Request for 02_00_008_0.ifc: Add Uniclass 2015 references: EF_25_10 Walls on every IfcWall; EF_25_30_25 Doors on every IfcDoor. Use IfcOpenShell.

First a look at what the model holds.

```python
import ifcopenshell

model = ifcopenshell.open("02_00_008_0.ifc")
print(model.schema)
print("classifications:", [c.Name for c in model.by_type("IfcClassification")])
for ifc_class in ("IfcDoor", "IfcRoof", "IfcStair", "IfcWall", "IfcWindow"):
    print(ifc_class, len(model.by_type(ifc_class)))
```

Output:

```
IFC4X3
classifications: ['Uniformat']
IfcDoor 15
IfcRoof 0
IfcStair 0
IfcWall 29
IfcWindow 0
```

```python
import ifcopenshell
import ifcopenshell.api.classification

model = ifcopenshell.open("02_00_008_0.ifc")

system = ifcopenshell.api.classification.add_classification(model, classification="Uniclass 2015")

codes = {
    "IfcWall": ("EF_25_10", "Walls"),
    "IfcDoor": ("EF_25_30_25", "Doors"),
}
for ifc_class, (code, name) in codes.items():
    products = model.by_type(ifc_class)
    ifcopenshell.api.classification.add_reference(
        model, products=products, classification=system, identification=code, name=name
    )
    print(code, len(products))

model.write("02_00_008_0_edited.ifc")
```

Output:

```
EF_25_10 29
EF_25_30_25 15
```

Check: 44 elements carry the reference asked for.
